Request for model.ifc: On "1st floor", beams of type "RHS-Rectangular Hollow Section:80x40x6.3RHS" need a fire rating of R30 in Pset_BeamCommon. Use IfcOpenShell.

First a look at what the model holds.

```python
import ifcopenshell
import ifcopenshell.util.element

model = ifcopenshell.open("model.ifc")
print(model.schema)
storey = next(s for s in model.by_type("IfcBuildingStorey") if s.Name == "1st floor")
beams = [e for e in ifcopenshell.util.element.get_decomposition(storey) if e.is_a("IfcBeam")]
seen = {}
for e in beams:
    element_type = ifcopenshell.util.element.get_type(e)
    key = (element_type.Name if element_type != e and element_type else None, ifcopenshell.util.element.get_pset(e, "Pset_BeamCommon", "FireRating"))
    seen[key] = seen.get(key, 0) + 1
for (name, value), count in sorted(seen.items(), key=str):
    print(count, "x", name, "|", value)
```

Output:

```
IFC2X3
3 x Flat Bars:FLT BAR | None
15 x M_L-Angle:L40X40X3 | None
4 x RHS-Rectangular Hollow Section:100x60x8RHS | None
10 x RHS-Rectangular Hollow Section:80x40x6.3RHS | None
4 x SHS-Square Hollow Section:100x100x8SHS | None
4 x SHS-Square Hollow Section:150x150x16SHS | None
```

```python
import ifcopenshell
import ifcopenshell.api.pset
import ifcopenshell.util.element

model = ifcopenshell.open("model.ifc")

storey = next(s for s in model.by_type("IfcBuildingStorey") if s.Name == "1st floor")
beams = [e for e in ifcopenshell.util.element.get_decomposition(storey) if e.is_a("IfcBeam")]

count = 0
for e in beams:
    element_type = ifcopenshell.util.element.get_type(e)
    if element_type in (None, e) or element_type.Name != "RHS-Rectangular Hollow Section:80x40x6.3RHS":
        continue
    # add_pset returns the element's existing set when there is one.
    pset = ifcopenshell.api.pset.add_pset(model, product=e, name="Pset_BeamCommon")
    ifcopenshell.api.pset.edit_pset(model, pset=pset, properties={"FireRating": "R30"})
    count += 1

print(count, "beams updated")

model.write("model_v2.ifc")
```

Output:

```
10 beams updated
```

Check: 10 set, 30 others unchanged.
